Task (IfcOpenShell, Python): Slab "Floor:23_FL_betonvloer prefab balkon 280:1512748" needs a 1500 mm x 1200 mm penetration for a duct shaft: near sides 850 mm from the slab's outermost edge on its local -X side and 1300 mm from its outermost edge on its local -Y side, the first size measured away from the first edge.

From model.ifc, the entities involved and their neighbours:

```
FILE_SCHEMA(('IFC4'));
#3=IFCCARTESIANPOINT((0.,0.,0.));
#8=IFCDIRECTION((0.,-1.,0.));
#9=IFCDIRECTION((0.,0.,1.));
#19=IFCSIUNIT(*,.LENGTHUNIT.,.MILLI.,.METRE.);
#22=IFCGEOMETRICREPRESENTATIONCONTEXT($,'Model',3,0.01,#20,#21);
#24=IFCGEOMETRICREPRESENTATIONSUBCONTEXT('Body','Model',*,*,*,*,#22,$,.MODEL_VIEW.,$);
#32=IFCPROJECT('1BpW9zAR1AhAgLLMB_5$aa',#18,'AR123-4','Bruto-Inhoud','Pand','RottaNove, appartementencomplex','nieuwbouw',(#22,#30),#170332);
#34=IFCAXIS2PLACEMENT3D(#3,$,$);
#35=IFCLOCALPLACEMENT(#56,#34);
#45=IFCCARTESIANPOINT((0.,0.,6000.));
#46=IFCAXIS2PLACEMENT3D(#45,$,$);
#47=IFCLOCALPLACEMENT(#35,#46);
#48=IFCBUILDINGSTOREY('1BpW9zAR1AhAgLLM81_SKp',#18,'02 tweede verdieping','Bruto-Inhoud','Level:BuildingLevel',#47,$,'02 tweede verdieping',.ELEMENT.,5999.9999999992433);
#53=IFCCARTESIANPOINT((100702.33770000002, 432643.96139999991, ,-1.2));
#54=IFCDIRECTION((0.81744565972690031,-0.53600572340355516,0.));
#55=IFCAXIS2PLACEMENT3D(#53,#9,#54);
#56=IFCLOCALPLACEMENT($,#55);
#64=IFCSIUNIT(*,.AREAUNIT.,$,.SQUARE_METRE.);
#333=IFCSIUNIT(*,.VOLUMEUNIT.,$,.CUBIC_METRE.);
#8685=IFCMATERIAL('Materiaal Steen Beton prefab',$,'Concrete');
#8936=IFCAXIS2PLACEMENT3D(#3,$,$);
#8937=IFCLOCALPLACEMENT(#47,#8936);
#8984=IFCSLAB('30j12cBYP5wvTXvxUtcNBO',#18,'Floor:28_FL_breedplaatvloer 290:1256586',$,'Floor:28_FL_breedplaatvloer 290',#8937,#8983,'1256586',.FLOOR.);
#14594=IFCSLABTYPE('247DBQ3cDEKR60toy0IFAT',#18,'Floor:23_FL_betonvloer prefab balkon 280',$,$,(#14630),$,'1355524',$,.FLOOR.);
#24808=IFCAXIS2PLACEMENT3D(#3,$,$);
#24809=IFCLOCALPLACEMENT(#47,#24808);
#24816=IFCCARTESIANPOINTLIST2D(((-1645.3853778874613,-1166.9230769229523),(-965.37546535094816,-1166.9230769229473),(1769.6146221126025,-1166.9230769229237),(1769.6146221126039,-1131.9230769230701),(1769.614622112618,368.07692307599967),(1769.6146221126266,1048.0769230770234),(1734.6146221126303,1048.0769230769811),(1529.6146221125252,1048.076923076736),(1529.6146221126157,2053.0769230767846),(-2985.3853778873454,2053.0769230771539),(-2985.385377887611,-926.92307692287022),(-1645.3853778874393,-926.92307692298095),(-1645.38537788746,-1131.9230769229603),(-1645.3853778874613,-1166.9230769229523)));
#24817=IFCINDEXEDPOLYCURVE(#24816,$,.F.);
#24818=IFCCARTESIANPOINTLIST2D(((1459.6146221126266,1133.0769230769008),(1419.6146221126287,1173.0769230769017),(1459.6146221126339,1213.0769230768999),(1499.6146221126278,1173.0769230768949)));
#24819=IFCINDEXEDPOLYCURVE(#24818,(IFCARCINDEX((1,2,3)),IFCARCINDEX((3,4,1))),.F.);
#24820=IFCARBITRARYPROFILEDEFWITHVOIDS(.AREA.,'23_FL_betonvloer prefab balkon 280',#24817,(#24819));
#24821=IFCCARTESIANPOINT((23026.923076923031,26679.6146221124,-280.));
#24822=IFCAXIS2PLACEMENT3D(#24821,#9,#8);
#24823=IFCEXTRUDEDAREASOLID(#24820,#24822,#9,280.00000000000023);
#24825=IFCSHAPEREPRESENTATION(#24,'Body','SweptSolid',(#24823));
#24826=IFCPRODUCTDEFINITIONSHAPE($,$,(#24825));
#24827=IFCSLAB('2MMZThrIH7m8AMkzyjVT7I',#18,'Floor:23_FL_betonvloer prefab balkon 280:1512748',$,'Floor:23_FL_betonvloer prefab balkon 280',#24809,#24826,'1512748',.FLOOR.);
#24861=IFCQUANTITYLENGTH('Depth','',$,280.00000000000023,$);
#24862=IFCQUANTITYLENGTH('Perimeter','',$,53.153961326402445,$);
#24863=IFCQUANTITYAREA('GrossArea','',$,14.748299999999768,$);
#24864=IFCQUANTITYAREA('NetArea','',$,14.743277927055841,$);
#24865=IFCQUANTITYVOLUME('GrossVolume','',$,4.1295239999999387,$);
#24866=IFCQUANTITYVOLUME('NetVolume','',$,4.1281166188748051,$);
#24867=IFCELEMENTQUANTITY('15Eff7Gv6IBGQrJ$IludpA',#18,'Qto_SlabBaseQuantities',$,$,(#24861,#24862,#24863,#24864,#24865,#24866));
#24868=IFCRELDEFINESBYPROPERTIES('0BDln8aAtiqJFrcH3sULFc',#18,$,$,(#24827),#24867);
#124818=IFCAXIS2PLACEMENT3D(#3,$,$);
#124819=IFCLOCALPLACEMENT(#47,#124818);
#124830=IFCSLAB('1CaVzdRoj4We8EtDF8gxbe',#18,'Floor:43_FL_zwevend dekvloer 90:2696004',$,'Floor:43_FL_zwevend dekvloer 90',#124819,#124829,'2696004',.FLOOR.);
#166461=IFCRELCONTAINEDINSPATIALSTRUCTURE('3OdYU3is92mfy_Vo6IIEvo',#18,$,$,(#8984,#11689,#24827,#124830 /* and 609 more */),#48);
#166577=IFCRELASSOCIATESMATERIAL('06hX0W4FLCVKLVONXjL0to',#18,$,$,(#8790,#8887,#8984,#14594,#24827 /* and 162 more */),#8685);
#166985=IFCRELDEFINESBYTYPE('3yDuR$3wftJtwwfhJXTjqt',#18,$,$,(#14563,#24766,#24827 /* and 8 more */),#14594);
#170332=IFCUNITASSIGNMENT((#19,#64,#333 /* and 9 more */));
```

```python
import numpy as np
import ifcopenshell
import ifcopenshell.api.feature
import ifcopenshell.api.geometry
import ifcopenshell.api.pset
import ifcopenshell.api.root
import ifcopenshell.geom
import ifcopenshell.util.element
import ifcopenshell.util.placement
import ifcopenshell.util.representation
import ifcopenshell.util.shape
import ifcopenshell.util.unit

model = ifcopenshell.open("model.ifc")
unit_scale = ifcopenshell.util.unit.calculate_unit_scale(model)
area_scale = ifcopenshell.util.unit.calculate_unit_scale(model, "AREAUNIT")
volume_scale = ifcopenshell.util.unit.calculate_unit_scale(model, "VOLUMEUNIT")
settings = ifcopenshell.geom.settings()


def volume(element):
    """Net volume in cubic metres, openings subtracted."""
    shape = ifcopenshell.geom.create_shape(settings, element)
    return ifcopenshell.util.shape.get_volume(shape.geometry)


slab = model.by_guid("2MMZThrIH7m8AMkzyjVT7I")
before = volume(slab)

# Extent in the slab's own axes, in metres. The edges named are its -X and -Y sides.
slab_shape = ifcopenshell.geom.create_shape(settings, slab)
vertices = ifcopenshell.util.shape.get_vertices(slab_shape.geometry)
x_min, y_min, bottom = vertices.min(axis=0)
top = vertices[:, 2].max()

opening = ifcopenshell.api.root.create_entity(model, ifc_class="IfcOpeningElement", name="Duct shaft opening", predefined_type="OPENING")
context = ifcopenshell.util.representation.get_context(model, "Model", "Body", "MODEL_VIEW")
width, depth = 1.5, 1.2
outline = [(0.0, 0.0), (width, 0.0), (width, depth), (0.0, depth), (0.0, 0.0)]
# Overshoot both faces by 50 mm so the cut is clean.
shape = ifcopenshell.api.geometry.add_slab_representation(
    model, context=context, depth=top - bottom + 0.1, polyline=outline
)
ifcopenshell.api.geometry.assign_representation(model, product=opening, representation=shape)

matrix = ifcopenshell.util.placement.get_local_placement(slab.ObjectPlacement)
matrix[:, 3] = matrix @ np.append(np.array([x_min + 0.85, y_min + 1.3, bottom - 0.05]) / unit_scale, 1.0)
ifcopenshell.api.geometry.edit_object_placement(model, product=opening, matrix=matrix, is_si=False)
ifcopenshell.api.feature.add_feature(model, feature=opening, element=slab)

after = volume(slab)

# Update the slab's stored quantities.
qto = model.by_id(ifcopenshell.util.element.get_pset(slab, "Qto_SlabBaseQuantities", should_inherit=False)["id"])
ifcopenshell.api.pset.edit_qto(model, qto=qto, properties={
    "NetArea": after / (top - bottom) / area_scale,
    "NetVolume": after / volume_scale,
})

print(f"slab volume {before:.3f} -> {after:.3f} m3")

model.write("model_edited.ifc")
```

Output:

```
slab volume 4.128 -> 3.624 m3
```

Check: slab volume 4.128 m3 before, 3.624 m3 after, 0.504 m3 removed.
